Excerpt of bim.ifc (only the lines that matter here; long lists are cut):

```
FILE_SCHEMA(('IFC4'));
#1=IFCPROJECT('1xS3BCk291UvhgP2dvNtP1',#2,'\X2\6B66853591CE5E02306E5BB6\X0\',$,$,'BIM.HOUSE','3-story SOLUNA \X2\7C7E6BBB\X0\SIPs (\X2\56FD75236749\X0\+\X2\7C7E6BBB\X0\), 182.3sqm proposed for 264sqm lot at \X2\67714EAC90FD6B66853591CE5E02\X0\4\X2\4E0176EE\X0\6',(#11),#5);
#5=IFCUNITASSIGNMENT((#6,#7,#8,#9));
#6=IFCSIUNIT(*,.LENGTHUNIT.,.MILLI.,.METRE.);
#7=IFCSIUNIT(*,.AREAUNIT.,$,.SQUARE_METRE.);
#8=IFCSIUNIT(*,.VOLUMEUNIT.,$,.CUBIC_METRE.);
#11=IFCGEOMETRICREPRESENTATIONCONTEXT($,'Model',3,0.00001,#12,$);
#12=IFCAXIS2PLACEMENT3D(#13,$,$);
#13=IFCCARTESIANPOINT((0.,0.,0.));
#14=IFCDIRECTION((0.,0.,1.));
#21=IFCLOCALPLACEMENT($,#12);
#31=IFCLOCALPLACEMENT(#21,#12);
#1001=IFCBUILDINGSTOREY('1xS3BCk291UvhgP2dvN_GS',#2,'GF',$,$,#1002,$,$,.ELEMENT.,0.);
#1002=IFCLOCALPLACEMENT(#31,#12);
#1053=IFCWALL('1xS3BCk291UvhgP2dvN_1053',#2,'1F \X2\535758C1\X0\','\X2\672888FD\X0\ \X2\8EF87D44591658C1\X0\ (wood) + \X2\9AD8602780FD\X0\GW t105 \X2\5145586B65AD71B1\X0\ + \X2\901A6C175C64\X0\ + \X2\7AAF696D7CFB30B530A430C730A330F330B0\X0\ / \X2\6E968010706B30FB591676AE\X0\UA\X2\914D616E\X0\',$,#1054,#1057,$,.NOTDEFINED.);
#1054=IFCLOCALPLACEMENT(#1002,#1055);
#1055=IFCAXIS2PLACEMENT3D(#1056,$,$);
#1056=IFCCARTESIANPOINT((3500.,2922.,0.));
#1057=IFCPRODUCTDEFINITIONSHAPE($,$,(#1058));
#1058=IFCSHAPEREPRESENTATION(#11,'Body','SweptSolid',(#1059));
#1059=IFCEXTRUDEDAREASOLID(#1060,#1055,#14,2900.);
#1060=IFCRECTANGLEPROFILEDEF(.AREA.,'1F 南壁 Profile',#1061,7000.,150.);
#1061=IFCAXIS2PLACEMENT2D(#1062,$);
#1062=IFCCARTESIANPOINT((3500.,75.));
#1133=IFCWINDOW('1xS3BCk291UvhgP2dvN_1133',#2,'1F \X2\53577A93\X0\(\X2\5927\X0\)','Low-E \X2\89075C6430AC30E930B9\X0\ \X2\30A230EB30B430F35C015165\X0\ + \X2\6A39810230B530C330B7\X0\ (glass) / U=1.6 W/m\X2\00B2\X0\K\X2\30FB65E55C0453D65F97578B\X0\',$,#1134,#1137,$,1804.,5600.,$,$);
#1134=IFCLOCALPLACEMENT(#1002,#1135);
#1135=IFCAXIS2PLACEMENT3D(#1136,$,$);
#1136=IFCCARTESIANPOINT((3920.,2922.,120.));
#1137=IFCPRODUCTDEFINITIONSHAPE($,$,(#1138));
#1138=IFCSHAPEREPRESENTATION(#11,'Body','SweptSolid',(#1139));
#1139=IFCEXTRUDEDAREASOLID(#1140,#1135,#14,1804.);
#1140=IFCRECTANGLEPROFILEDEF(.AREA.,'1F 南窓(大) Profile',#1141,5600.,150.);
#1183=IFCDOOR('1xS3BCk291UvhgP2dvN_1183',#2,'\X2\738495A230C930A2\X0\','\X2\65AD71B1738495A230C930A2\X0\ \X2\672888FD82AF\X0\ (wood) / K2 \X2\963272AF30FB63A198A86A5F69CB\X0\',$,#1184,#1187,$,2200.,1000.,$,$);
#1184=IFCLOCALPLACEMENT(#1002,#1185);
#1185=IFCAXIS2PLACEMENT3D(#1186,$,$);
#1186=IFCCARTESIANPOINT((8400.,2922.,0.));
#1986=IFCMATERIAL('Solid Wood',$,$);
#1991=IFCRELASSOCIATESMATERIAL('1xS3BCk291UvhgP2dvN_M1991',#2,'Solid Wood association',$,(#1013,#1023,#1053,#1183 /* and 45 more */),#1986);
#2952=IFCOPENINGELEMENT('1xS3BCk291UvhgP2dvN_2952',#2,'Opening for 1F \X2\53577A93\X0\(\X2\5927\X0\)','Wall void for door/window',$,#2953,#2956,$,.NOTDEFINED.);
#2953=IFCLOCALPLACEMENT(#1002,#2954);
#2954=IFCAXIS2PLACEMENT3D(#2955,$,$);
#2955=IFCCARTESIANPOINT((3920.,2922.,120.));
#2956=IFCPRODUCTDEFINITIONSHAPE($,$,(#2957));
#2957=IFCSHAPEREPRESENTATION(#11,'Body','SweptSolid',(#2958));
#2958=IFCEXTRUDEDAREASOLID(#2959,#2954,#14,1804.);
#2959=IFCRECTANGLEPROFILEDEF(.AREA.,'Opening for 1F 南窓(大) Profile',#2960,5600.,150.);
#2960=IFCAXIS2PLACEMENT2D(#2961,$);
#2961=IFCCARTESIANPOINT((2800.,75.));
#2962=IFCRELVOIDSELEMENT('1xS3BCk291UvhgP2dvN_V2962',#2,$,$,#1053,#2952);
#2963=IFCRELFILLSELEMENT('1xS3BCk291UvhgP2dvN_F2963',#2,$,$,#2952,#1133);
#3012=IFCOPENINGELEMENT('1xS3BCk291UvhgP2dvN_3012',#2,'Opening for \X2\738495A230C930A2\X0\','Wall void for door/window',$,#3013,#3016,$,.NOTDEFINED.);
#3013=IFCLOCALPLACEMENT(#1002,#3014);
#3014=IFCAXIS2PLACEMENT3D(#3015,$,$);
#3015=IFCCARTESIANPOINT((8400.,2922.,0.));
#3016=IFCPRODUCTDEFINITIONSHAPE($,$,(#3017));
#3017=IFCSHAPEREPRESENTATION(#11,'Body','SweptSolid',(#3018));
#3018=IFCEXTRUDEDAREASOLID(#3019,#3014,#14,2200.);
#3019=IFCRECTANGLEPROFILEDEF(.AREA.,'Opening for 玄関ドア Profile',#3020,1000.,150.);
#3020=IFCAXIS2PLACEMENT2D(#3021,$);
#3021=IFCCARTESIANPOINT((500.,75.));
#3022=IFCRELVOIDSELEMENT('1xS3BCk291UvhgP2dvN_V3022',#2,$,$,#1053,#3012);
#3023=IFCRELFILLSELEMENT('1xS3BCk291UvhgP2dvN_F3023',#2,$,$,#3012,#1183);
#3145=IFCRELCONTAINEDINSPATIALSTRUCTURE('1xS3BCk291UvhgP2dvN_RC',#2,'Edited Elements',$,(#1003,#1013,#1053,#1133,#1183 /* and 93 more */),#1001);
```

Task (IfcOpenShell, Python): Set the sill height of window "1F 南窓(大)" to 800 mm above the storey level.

```python
import numpy as np
import ifcopenshell
import ifcopenshell.api.geometry
import ifcopenshell.geom
import ifcopenshell.util.element
import ifcopenshell.util.placement
import ifcopenshell.util.shape
import ifcopenshell.util.unit

model = ifcopenshell.open("bim.ifc")
unit_scale = ifcopenshell.util.unit.calculate_unit_scale(model)

window = model.by_guid("1xS3BCk291UvhgP2dvN_1133")
opening = window.FillsVoids[0].RelatingOpeningElement
storey = ifcopenshell.util.element.get_container(window, ifc_class="IfcBuildingStorey")
level = ifcopenshell.util.placement.get_local_placement(storey.ObjectPlacement)[2, 3]

# The opening's origin need not be at the sill, so measure its lowest point.
shape = ifcopenshell.geom.create_shape(ifcopenshell.geom.settings(), opening)
bottom = ifcopenshell.util.shape.get_shape_bottom_elevation(shape, shape.geometry) / unit_scale
dz = level + 0.8 / unit_scale - bottom

shift = np.array([0.0, 0.0, dz])
# The window is not placed relative to its opening, so move both.
for product in (opening, window):
    matrix = ifcopenshell.util.placement.get_local_placement(product.ObjectPlacement)
    matrix[:3, 3] += shift
    ifcopenshell.api.geometry.edit_object_placement(model, product=product, matrix=matrix, is_si=False)

print(f"moved by {dz * unit_scale:+.3f} m")

model.write("bim_rev.ifc")
```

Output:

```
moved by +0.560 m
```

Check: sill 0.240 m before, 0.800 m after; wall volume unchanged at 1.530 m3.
